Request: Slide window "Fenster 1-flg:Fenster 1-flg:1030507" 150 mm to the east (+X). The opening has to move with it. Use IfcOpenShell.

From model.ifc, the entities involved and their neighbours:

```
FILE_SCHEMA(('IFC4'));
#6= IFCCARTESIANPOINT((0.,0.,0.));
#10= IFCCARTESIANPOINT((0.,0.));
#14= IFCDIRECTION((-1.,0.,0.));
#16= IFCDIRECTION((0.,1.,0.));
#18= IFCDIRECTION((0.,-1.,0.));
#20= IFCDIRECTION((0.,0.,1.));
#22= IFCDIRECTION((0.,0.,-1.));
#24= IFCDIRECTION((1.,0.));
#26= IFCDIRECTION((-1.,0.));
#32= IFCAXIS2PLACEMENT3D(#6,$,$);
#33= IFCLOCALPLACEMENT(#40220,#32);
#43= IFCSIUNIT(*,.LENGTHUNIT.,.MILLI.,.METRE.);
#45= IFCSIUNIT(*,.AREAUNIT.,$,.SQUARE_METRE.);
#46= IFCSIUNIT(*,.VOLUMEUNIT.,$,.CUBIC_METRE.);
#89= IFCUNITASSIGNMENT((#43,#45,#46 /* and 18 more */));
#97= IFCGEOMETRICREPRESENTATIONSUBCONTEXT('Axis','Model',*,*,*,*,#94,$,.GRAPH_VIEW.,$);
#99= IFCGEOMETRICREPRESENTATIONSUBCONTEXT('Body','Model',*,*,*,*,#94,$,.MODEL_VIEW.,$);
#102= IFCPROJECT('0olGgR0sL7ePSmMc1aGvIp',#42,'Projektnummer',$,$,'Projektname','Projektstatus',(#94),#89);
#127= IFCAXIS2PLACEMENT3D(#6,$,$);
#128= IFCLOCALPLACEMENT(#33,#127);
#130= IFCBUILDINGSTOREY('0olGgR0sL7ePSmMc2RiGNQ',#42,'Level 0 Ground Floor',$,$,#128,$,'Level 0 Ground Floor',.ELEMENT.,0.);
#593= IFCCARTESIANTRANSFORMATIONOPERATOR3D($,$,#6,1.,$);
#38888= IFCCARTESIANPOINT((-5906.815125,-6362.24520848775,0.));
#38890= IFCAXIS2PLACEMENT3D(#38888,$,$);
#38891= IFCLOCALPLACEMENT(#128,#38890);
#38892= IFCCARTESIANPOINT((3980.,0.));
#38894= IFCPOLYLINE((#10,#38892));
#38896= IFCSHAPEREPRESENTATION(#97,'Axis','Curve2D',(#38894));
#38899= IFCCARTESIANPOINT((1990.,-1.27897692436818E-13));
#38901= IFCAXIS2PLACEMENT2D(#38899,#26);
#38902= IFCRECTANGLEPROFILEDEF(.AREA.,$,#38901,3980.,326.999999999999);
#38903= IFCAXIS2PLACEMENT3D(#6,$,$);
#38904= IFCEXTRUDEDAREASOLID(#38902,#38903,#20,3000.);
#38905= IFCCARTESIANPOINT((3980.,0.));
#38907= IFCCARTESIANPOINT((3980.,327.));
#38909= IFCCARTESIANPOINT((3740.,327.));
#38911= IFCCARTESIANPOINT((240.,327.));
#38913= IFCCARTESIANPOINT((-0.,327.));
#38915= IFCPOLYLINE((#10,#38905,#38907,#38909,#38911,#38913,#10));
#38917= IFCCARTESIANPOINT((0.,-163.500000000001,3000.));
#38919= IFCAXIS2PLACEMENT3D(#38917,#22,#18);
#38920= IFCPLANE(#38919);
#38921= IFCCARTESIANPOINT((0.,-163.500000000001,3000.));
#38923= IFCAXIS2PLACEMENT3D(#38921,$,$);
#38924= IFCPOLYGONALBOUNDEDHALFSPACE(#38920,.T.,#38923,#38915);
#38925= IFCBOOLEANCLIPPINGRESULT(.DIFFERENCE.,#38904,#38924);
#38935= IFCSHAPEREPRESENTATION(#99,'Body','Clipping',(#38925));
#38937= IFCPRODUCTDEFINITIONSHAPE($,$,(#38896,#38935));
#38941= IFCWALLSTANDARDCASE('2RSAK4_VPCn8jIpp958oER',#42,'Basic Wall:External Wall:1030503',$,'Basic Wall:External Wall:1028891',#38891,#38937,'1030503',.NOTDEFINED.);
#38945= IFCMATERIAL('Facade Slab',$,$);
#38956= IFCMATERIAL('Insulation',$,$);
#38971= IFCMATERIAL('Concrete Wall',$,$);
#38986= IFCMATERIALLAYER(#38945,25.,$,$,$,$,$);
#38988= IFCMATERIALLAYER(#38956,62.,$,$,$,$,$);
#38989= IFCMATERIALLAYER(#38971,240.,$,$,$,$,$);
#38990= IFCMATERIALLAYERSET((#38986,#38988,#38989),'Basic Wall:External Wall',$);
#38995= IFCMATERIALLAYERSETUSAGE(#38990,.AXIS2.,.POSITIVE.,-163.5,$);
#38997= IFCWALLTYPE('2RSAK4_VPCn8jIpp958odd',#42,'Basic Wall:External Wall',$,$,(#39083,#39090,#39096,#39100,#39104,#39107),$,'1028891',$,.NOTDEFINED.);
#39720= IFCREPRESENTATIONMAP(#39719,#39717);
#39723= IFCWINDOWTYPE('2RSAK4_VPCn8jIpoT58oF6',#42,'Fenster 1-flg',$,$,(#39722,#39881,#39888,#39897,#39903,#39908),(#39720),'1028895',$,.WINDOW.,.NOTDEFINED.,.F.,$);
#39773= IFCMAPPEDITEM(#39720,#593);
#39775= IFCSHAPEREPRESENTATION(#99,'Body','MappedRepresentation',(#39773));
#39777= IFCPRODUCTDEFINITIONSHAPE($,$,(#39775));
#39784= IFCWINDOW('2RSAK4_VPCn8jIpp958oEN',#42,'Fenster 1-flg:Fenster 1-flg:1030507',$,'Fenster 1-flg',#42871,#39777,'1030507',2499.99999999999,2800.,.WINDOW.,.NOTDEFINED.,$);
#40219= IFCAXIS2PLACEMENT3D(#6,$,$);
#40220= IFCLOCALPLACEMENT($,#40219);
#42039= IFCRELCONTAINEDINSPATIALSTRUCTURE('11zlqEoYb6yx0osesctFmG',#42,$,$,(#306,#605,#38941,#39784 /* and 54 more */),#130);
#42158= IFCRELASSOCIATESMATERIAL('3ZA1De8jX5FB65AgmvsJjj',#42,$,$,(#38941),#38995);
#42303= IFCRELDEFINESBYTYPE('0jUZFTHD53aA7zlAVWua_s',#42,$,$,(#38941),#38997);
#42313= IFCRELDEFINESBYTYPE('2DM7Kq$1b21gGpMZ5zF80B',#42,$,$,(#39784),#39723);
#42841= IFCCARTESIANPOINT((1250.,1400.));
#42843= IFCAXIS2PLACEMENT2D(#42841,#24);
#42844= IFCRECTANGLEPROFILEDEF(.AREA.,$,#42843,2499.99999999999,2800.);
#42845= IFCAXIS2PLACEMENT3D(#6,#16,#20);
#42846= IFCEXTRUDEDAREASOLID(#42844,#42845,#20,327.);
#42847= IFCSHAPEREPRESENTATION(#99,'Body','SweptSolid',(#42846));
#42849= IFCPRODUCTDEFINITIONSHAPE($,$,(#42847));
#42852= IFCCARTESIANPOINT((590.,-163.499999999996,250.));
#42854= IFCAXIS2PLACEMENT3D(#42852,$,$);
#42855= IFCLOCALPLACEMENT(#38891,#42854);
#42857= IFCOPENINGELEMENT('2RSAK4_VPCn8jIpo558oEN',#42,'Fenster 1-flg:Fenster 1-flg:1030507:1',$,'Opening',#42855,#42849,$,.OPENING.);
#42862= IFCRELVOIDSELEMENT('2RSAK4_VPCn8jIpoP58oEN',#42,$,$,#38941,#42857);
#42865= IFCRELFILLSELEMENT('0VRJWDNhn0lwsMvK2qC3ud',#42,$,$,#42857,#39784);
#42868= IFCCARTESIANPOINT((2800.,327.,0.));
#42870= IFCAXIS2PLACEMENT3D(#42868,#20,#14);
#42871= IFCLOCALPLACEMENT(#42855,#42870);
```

```python
import ifcopenshell
import ifcopenshell.api.geometry
import ifcopenshell.util.placement
import ifcopenshell.util.unit

model = ifcopenshell.open("model.ifc")
unit_scale = ifcopenshell.util.unit.calculate_unit_scale(model)

window = model.by_guid("2RSAK4_VPCn8jIpp958oEN")
opening = window.FillsVoids[0].RelatingOpeningElement
wall = opening.VoidsElements[0].RelatingBuildingElement

wall_matrix = ifcopenshell.util.placement.get_local_placement(wall.ObjectPlacement)
shift = wall_matrix[:3, 0] * 0.15 / unit_scale
before = ifcopenshell.util.placement.get_local_placement(window.ObjectPlacement)[:3, 3].copy()

# The window is placed relative to its opening, so it follows when the opening moves.
matrix = ifcopenshell.util.placement.get_local_placement(opening.ObjectPlacement)
matrix[:3, 3] += shift
ifcopenshell.api.geometry.edit_object_placement(
    model, product=opening, matrix=matrix, is_si=False, should_transform_children=True
)

after = ifcopenshell.util.placement.get_local_placement(window.ObjectPlacement)[:3, 3]
print("window moved by", (after - before).round(3) + 0.0)

model.write("model_rev.ifc")
```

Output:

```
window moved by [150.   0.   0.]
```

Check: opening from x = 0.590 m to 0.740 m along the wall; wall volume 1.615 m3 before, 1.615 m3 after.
